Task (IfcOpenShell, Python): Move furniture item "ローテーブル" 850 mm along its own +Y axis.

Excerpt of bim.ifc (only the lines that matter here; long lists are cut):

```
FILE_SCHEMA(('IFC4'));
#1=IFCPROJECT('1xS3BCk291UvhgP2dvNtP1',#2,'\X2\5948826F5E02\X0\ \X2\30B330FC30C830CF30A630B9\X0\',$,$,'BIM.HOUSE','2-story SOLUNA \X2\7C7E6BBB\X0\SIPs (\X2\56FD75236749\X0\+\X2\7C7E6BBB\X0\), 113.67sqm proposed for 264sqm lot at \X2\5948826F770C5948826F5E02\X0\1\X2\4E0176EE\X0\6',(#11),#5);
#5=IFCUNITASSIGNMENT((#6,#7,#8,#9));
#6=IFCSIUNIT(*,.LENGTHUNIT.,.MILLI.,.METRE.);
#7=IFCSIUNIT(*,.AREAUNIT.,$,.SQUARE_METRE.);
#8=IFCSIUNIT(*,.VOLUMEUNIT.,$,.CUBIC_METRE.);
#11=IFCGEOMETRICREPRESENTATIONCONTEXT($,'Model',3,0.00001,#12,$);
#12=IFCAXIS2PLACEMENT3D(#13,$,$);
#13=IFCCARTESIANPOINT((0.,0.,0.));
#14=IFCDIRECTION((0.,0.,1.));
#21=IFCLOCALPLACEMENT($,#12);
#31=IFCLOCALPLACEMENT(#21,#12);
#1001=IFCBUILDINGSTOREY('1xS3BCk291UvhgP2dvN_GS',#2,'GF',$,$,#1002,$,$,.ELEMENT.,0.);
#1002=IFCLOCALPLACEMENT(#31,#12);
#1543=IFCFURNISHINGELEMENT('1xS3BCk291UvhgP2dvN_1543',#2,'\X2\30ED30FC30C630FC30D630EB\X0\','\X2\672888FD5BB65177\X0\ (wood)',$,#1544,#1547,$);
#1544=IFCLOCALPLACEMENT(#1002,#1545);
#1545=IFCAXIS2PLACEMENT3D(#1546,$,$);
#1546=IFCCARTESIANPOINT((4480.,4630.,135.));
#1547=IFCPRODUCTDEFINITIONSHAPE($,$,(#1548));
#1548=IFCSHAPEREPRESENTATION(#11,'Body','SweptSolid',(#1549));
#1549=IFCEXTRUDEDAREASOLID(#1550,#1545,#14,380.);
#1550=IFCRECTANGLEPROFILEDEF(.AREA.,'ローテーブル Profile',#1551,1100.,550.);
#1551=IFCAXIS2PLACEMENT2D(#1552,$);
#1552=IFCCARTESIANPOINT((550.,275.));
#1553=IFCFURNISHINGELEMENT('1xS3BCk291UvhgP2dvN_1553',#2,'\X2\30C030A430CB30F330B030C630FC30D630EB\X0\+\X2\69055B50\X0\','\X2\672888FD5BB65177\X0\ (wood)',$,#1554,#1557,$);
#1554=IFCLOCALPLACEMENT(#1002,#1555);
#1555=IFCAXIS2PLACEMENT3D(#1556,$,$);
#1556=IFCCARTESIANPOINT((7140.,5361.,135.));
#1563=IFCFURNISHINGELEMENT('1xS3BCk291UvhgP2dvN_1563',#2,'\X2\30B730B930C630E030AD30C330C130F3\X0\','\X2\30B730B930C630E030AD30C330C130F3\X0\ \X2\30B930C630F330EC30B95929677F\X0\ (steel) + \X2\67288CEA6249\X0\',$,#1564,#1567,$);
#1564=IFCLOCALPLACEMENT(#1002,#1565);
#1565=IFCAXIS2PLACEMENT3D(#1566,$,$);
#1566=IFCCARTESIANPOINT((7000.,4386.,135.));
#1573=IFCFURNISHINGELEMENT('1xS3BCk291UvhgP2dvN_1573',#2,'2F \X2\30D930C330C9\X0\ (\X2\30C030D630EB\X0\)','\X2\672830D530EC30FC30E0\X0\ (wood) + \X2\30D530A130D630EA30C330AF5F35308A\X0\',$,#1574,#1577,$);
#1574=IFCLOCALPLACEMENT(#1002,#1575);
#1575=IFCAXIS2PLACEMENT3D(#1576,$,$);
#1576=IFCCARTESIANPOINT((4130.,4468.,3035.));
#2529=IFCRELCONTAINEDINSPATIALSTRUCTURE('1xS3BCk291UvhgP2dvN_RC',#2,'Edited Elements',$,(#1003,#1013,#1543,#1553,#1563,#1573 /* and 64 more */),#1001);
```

```python
import ifcopenshell
import ifcopenshell.api.geometry
import ifcopenshell.util.placement
import ifcopenshell.util.unit

model = ifcopenshell.open("bim.ifc")
unit_scale = ifcopenshell.util.unit.calculate_unit_scale(model)

item = model.by_guid("1xS3BCk291UvhgP2dvN_1543")
matrix = ifcopenshell.util.placement.get_local_placement(item.ObjectPlacement)
matrix[:3, 3] += matrix[:3, 1] * 0.85 / unit_scale
ifcopenshell.api.geometry.edit_object_placement(model, product=item, matrix=matrix, is_si=False)

print(ifcopenshell.util.placement.get_local_placement(item.ObjectPlacement).round(3) + 0.0)

model.write("bim-out.ifc")
```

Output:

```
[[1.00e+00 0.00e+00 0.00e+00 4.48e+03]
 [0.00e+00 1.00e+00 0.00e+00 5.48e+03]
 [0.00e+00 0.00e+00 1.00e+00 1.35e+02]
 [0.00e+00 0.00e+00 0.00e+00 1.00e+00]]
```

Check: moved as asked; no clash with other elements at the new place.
